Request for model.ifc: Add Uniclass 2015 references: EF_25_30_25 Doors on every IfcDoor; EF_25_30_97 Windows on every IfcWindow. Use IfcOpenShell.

First a look at what the model holds.

```python
import ifcopenshell

model = ifcopenshell.open("model.ifc")
print(model.schema)
print("classifications:", [c.Name for c in model.by_type("IfcClassification")])
for ifc_class in ("IfcDoor", "IfcRoof", "IfcStair", "IfcWall", "IfcWindow"):
    print(ifc_class, len(model.by_type(ifc_class)))
```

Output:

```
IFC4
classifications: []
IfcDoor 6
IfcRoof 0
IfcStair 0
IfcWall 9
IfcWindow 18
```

```python
import ifcopenshell
import ifcopenshell.api.classification

model = ifcopenshell.open("model.ifc")

system = ifcopenshell.api.classification.add_classification(model, classification="Uniclass 2015")

codes = {
    "IfcDoor": ("EF_25_30_25", "Doors"),
    "IfcWindow": ("EF_25_30_97", "Windows"),
}
for ifc_class, (code, name) in codes.items():
    products = model.by_type(ifc_class)
    ifcopenshell.api.classification.add_reference(
        model, products=products, classification=system, identification=code, name=name
    )
    print(code, len(products))

model.write("model_v2.ifc")
```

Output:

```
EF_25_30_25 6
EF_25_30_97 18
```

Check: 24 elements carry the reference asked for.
